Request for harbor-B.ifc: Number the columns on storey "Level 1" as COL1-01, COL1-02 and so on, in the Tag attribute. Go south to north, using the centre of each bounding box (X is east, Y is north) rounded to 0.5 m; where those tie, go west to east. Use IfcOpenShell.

First a look at what the model holds.

```python
import ifcopenshell
import ifcopenshell.util.element
import ifcopenshell.util.placement

model = ifcopenshell.open("harbor-B.ifc")
print(model.schema)
storey = next(s for s in model.by_type("IfcBuildingStorey") if s.Name == "Level 1")
columns = [e for e in ifcopenshell.util.element.get_decomposition(storey) if e.is_a("IfcColumn")]
for e in sorted(columns, key=lambda e: e.id()):
    origin = ifcopenshell.util.placement.get_local_placement(e.ObjectPlacement)[:3, 3]
    print(e.id(), e.Tag, e.Name, origin.round(2) + 0.0, sep=" | ")
```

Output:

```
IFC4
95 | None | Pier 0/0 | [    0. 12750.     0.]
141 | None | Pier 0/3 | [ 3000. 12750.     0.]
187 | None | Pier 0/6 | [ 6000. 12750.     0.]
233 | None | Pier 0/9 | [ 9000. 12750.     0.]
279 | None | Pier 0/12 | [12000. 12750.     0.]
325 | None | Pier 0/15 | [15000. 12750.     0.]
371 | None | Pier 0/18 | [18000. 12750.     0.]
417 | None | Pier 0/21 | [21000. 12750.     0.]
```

```python
import ifcopenshell
import ifcopenshell.geom
import ifcopenshell.util.element
import ifcopenshell.util.shape

model = ifcopenshell.open("harbor-B.ifc")
settings = ifcopenshell.geom.settings()
settings.set("use-world-coords", True)


def centre(element):
    shape = ifcopenshell.geom.create_shape(settings, element)
    return ifcopenshell.util.shape.get_bbox_centroid(shape.geometry)


storey = next(s for s in model.by_type("IfcBuildingStorey") if s.Name == "Level 1")
columns = [e for e in ifcopenshell.util.element.get_decomposition(storey) if e.is_a("IfcColumn")]

# Insertion points can sit at a corner or the storey origin, so sort by the geometry (in metres).
centres = {e: centre(e) for e in columns}
columns.sort(key=lambda e: (round(centres[e][1] / 0.5), centres[e][0]))

for i, e in enumerate(columns, start=1):
    number = f"COL1-{i:02d}"
    e.Tag = number
    print(e.id(), number)

model.write("harbor-B_v2.ifc")
```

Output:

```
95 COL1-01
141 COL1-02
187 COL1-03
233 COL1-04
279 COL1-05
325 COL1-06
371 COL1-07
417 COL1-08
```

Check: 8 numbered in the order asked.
